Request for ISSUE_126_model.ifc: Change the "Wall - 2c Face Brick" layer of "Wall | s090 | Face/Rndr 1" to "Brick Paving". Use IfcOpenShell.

First a look at what the model holds.

```python
import ifcopenshell
import ifcopenshell.util.element

model = ifcopenshell.open("ISSUE_126_model.ifc")
print(model.schema)
for layer_set in model.by_type("IfcMaterialLayerSet"):
    if layer_set.LayerSetName == "Wall | s090 | Face/Rndr 1":
        for layer in layer_set.MaterialLayers:
            print(layer.id(), layer.Material and layer.Material.Name, layer.LayerThickness, sep=" | ")
        print(len(ifcopenshell.util.element.get_elements_by_material(model, layer_set)), "elements and types use it")
print(sorted(m.Name for m in model.by_type("IfcMaterial") if m.Name)[:60])
```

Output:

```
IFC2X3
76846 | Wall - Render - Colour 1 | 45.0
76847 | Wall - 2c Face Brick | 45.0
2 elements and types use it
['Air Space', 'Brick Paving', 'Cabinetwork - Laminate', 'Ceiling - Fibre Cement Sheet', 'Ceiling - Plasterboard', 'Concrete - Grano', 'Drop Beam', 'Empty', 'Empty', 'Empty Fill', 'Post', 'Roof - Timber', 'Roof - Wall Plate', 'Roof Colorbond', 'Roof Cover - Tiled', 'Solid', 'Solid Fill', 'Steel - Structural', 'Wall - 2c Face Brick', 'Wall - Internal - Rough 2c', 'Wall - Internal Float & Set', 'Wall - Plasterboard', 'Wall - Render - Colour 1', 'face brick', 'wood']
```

```python
import ifcopenshell
import ifcopenshell.api.material

model = ifcopenshell.open("ISSUE_126_model.ifc")

layer_set = next(s for s in model.by_type("IfcMaterialLayerSet") if s.LayerSetName == "Wall | s090 | Face/Rndr 1")
layer = next(l for l in layer_set.MaterialLayers if l.Material and l.Material.Name == "Wall - 2c Face Brick")
material = next(m for m in model.by_type("IfcMaterial") if m.Name == "Brick Paving")

# Point this one layer at the other material; renaming the old one would change it everywhere.
ifcopenshell.api.material.edit_layer(model, layer=layer, attributes={}, material=material)

print([l.Material.Name if l.Material else None for l in layer_set.MaterialLayers])

model.write("ISSUE_126_model_rev.ifc")
```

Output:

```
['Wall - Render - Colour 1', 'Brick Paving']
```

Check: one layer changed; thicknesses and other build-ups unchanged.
